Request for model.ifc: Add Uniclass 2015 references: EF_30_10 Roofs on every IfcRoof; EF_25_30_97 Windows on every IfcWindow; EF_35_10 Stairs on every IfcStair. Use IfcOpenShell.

First a look at what the model holds.

```python
import ifcopenshell

model = ifcopenshell.open("model.ifc")
print(model.schema)
print("classifications:", [c.Name for c in model.by_type("IfcClassification")])
for ifc_class in ("IfcDoor", "IfcRoof", "IfcStair", "IfcWall", "IfcWindow"):
    print(ifc_class, len(model.by_type(ifc_class)))
```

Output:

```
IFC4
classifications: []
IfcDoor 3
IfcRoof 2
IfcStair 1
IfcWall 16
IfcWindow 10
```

```python
import ifcopenshell
import ifcopenshell.api.classification

model = ifcopenshell.open("model.ifc")

system = ifcopenshell.api.classification.add_classification(model, classification="Uniclass 2015")

codes = {
    "IfcRoof": ("EF_30_10", "Roofs"),
    "IfcWindow": ("EF_25_30_97", "Windows"),
    "IfcStair": ("EF_35_10", "Stairs"),
}
for ifc_class, (code, name) in codes.items():
    products = model.by_type(ifc_class)
    ifcopenshell.api.classification.add_reference(
        model, products=products, classification=system, identification=code, name=name
    )
    print(code, len(products))

model.write("model_edited.ifc")
```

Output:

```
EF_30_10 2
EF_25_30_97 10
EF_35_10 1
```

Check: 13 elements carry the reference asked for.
